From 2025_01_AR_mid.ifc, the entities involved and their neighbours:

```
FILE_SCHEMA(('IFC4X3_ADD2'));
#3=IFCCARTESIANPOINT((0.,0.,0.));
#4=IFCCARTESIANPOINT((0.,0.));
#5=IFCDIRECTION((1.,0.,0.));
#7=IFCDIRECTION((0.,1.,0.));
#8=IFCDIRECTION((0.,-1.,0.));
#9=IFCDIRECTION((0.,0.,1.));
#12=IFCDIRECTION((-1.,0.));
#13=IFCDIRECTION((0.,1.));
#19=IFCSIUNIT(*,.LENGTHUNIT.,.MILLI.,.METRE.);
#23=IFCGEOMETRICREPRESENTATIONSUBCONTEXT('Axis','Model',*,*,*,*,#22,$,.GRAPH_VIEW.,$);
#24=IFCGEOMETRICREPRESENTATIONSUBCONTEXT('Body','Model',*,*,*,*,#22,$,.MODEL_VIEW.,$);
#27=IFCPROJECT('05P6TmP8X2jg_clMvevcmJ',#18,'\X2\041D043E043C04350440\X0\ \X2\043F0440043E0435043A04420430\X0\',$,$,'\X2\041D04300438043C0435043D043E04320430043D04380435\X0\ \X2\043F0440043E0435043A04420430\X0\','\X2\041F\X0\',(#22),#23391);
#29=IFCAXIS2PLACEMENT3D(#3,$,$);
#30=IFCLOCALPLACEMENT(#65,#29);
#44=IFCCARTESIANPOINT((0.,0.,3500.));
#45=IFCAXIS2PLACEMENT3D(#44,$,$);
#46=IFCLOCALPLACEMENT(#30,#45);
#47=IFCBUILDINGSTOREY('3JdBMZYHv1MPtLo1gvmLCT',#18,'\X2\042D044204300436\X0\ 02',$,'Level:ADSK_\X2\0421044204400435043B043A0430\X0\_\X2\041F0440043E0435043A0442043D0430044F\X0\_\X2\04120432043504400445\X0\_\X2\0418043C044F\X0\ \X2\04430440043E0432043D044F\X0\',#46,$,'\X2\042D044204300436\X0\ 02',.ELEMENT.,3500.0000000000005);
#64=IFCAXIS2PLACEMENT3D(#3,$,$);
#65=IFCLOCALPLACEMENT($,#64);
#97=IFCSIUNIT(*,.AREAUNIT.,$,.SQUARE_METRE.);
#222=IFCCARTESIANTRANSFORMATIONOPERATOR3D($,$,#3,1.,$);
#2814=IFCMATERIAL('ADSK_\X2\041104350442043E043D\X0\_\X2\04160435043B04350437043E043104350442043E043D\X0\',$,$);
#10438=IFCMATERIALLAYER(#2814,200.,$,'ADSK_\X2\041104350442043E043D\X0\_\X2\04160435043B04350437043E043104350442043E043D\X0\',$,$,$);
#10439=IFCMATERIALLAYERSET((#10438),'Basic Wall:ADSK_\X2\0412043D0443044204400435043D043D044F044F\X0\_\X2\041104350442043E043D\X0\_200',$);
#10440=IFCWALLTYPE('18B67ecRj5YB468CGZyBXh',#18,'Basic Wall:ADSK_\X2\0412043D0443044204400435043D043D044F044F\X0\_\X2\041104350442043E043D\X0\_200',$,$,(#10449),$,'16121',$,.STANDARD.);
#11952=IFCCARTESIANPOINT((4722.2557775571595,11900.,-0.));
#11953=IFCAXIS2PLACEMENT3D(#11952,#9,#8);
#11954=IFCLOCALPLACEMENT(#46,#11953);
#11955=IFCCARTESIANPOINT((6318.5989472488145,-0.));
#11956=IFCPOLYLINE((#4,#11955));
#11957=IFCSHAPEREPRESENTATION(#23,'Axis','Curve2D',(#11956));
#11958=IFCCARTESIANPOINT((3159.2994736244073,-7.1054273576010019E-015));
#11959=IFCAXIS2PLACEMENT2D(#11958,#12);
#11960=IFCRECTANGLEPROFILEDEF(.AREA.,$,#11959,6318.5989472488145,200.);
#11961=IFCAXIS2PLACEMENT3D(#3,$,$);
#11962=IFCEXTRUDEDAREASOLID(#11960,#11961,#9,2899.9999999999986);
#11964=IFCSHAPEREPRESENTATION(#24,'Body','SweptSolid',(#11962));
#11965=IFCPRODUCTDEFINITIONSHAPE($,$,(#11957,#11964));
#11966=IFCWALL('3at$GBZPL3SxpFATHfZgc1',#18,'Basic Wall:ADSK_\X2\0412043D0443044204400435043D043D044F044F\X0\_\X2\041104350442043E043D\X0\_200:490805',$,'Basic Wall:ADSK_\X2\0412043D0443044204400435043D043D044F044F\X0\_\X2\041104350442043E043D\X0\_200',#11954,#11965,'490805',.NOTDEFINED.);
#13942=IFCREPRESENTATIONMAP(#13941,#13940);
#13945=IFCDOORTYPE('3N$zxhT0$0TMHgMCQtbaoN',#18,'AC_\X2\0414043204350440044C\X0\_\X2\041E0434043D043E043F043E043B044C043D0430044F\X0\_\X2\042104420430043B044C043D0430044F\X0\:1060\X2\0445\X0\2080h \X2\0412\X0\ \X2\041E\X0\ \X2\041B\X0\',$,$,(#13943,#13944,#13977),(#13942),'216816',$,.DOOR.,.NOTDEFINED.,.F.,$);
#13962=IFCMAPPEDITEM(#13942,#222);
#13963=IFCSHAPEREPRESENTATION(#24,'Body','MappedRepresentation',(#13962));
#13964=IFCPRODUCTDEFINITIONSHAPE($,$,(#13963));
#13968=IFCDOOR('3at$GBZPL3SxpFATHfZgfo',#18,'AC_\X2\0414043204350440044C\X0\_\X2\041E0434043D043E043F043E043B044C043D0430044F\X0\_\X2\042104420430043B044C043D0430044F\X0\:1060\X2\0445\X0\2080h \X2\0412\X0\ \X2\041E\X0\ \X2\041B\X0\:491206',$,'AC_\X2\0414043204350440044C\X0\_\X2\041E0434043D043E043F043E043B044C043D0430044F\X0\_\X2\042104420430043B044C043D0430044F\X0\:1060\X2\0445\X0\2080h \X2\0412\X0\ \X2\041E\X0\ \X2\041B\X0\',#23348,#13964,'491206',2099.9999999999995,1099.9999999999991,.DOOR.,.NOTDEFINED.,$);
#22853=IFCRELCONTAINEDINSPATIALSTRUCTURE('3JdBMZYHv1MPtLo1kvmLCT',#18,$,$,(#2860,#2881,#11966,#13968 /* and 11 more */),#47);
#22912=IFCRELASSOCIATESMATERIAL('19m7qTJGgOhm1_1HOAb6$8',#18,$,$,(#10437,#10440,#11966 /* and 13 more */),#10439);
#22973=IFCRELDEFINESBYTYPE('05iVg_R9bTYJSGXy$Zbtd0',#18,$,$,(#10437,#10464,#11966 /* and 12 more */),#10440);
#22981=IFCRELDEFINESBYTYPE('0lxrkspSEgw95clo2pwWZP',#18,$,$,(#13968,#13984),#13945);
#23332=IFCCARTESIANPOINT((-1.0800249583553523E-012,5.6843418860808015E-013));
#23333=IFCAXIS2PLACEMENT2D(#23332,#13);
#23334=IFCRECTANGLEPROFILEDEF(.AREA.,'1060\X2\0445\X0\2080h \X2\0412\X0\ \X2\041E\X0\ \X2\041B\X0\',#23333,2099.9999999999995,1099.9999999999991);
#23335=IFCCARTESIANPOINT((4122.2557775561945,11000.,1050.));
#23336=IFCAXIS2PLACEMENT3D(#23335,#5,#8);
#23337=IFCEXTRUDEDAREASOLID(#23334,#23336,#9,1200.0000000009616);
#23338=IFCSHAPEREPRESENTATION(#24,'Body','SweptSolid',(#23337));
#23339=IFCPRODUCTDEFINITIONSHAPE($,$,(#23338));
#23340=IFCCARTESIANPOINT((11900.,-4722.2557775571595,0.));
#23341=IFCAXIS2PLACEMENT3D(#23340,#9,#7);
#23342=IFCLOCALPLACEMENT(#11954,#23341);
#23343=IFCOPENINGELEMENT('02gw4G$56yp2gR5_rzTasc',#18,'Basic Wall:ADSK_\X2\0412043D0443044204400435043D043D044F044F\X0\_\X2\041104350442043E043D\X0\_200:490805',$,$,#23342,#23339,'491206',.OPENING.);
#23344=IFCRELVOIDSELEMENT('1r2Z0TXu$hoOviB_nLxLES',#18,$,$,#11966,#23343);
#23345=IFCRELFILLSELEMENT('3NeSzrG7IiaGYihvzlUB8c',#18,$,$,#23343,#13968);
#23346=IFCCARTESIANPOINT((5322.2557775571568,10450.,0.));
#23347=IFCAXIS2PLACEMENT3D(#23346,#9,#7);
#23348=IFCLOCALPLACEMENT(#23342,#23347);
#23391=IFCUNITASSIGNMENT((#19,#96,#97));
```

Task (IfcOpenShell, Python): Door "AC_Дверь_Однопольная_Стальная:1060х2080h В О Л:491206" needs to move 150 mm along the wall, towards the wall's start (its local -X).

```python
import ifcopenshell
import ifcopenshell.api.geometry
import ifcopenshell.util.placement
import ifcopenshell.util.unit

model = ifcopenshell.open("2025_01_AR_mid.ifc")
unit_scale = ifcopenshell.util.unit.calculate_unit_scale(model)

door = model.by_id(13968)
opening = door.FillsVoids[0].RelatingOpeningElement
wall = opening.VoidsElements[0].RelatingBuildingElement

wall_matrix = ifcopenshell.util.placement.get_local_placement(wall.ObjectPlacement)
shift = wall_matrix[:3, 0] * -0.15 / unit_scale
before = ifcopenshell.util.placement.get_local_placement(door.ObjectPlacement)[:3, 3].copy()

# The door is placed relative to its opening, so it follows when the opening moves.
matrix = ifcopenshell.util.placement.get_local_placement(opening.ObjectPlacement)
matrix[:3, 3] += shift
ifcopenshell.api.geometry.edit_object_placement(
    model, product=opening, matrix=matrix, is_si=False, should_transform_children=True
)

after = ifcopenshell.util.placement.get_local_placement(door.ObjectPlacement)[:3, 3]
print("door moved by", (after - before).round(3) + 0.0)

model.write("2025_01_AR_mid_rev.ifc")
```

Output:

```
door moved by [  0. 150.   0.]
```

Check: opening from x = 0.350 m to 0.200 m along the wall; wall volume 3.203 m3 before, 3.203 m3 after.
